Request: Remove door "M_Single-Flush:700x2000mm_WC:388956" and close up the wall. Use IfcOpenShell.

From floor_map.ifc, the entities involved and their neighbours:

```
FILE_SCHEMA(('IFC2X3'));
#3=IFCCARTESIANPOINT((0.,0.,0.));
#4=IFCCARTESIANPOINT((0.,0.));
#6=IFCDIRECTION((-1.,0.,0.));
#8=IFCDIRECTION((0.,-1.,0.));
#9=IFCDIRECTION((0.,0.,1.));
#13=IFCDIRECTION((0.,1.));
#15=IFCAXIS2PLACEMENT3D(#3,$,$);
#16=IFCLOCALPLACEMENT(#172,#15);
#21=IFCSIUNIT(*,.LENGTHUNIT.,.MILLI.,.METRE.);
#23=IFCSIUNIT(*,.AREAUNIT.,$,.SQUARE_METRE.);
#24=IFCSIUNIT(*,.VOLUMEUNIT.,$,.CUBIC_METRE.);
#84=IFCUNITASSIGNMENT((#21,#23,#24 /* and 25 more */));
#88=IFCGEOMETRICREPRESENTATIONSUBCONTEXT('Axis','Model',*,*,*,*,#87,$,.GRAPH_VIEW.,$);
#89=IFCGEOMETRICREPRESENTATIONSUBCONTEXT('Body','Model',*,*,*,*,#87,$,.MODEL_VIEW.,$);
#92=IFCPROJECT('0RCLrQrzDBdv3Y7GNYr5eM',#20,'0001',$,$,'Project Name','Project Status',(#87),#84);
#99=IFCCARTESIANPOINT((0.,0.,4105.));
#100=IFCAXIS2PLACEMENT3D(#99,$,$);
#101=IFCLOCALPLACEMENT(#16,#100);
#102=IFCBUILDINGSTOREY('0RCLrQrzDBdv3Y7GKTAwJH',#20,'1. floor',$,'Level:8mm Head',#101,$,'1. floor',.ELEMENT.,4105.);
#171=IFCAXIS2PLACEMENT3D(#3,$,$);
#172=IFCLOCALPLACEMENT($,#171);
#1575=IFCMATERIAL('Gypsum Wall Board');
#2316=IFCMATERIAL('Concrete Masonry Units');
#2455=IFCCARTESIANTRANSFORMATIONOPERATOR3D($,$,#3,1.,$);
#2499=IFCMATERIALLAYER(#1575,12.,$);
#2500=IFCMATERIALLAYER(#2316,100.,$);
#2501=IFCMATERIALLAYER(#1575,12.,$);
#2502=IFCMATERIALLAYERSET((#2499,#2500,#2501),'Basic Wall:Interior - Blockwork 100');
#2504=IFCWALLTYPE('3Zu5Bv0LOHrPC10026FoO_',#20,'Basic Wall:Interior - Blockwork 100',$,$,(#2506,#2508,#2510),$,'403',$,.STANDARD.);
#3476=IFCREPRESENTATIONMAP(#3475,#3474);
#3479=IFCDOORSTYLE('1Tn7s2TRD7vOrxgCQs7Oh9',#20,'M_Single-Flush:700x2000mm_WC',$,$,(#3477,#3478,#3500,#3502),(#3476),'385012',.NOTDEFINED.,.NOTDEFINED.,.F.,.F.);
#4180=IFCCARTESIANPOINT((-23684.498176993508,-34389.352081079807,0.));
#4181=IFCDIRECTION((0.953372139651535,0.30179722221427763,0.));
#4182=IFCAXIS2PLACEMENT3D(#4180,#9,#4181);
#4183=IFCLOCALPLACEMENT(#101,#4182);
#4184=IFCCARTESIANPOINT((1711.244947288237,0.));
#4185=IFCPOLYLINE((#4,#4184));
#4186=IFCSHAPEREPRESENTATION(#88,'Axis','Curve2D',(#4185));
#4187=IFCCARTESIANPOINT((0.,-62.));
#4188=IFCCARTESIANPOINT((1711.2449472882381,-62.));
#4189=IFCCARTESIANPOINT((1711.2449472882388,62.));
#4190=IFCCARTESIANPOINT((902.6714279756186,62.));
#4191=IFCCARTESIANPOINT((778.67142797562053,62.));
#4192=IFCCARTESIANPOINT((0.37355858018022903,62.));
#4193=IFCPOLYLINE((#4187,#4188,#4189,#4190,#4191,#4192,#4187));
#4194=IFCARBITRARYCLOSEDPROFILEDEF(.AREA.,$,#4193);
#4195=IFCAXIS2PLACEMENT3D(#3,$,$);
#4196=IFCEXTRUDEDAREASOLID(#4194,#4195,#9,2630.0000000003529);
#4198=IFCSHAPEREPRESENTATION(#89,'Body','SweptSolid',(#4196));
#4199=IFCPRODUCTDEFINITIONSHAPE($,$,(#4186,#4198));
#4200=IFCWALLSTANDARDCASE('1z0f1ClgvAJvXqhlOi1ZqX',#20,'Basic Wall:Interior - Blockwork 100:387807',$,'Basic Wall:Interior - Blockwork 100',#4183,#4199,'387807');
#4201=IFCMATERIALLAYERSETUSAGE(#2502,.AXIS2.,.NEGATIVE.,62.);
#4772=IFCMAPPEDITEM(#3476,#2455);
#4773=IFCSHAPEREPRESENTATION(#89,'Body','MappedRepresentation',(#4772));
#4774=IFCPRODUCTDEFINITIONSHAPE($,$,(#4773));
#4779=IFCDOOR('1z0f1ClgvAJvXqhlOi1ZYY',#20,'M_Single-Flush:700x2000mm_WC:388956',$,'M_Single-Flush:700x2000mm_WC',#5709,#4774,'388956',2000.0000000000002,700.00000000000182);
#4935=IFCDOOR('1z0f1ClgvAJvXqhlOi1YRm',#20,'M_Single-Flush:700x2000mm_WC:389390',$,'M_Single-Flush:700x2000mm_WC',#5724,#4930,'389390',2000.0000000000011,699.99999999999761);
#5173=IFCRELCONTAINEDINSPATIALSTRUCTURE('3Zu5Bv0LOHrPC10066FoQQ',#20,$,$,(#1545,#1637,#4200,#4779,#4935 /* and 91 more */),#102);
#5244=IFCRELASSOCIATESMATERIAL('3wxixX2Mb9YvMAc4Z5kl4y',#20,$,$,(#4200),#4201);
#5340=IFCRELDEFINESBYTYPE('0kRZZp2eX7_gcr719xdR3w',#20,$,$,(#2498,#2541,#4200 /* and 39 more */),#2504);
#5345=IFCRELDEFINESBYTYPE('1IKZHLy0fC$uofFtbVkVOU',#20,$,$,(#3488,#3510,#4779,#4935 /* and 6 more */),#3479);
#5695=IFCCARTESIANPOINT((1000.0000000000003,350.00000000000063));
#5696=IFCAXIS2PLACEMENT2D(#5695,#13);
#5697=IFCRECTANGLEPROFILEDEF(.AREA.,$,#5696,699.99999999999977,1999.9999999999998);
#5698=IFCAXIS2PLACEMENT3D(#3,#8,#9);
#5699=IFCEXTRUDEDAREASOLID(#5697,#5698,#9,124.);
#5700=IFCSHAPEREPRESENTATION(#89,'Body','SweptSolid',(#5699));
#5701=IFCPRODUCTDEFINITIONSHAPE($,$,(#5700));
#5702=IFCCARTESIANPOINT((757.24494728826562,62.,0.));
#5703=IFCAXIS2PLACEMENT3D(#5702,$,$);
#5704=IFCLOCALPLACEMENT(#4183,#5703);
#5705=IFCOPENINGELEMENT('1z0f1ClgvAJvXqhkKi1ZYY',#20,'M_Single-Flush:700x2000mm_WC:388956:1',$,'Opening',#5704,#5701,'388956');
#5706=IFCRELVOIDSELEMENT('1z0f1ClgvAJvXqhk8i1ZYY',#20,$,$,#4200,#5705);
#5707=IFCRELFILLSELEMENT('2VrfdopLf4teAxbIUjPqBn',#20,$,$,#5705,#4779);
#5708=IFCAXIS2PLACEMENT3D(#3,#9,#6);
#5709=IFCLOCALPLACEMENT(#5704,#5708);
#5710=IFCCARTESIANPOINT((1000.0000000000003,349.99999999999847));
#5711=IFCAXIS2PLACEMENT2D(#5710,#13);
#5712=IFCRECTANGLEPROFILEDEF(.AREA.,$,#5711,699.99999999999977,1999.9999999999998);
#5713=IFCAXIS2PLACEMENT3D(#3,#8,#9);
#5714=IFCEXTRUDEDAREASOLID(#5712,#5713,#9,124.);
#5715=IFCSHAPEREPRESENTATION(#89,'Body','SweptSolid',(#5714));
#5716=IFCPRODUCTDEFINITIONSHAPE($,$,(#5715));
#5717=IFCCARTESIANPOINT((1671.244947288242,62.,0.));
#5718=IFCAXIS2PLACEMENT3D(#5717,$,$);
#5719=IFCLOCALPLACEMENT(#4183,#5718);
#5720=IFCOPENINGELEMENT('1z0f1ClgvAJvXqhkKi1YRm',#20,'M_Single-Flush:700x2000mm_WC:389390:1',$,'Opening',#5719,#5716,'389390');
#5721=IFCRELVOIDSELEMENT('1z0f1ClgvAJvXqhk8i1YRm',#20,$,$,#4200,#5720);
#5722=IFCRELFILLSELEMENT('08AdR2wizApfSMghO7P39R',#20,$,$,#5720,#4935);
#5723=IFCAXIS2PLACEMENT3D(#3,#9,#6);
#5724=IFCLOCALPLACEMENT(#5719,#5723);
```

```python
import ifcopenshell
import ifcopenshell.api.feature
import ifcopenshell.api.root
import ifcopenshell.geom
import ifcopenshell.util.shape

model = ifcopenshell.open("floor_map.ifc")
settings = ifcopenshell.geom.settings()


def volume(element):
    """Net volume in cubic metres, openings subtracted."""
    shape = ifcopenshell.geom.create_shape(settings, element)
    return ifcopenshell.util.shape.get_volume(shape.geometry)


door = model.by_guid("1z0f1ClgvAJvXqhlOi1ZYY")
opening = door.FillsVoids[0].RelatingOpeningElement
wall = opening.VoidsElements[0].RelatingBuildingElement
before = volume(wall)

ifcopenshell.api.root.remove_product(model, product=door)
ifcopenshell.api.feature.remove_feature(model, feature=opening)

after = volume(wall)

print(f"wall volume {before:.3f} -> {after:.3f} m3")

model.write("floor_map-out.ifc")
```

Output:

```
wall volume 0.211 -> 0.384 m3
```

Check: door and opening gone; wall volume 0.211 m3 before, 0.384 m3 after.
